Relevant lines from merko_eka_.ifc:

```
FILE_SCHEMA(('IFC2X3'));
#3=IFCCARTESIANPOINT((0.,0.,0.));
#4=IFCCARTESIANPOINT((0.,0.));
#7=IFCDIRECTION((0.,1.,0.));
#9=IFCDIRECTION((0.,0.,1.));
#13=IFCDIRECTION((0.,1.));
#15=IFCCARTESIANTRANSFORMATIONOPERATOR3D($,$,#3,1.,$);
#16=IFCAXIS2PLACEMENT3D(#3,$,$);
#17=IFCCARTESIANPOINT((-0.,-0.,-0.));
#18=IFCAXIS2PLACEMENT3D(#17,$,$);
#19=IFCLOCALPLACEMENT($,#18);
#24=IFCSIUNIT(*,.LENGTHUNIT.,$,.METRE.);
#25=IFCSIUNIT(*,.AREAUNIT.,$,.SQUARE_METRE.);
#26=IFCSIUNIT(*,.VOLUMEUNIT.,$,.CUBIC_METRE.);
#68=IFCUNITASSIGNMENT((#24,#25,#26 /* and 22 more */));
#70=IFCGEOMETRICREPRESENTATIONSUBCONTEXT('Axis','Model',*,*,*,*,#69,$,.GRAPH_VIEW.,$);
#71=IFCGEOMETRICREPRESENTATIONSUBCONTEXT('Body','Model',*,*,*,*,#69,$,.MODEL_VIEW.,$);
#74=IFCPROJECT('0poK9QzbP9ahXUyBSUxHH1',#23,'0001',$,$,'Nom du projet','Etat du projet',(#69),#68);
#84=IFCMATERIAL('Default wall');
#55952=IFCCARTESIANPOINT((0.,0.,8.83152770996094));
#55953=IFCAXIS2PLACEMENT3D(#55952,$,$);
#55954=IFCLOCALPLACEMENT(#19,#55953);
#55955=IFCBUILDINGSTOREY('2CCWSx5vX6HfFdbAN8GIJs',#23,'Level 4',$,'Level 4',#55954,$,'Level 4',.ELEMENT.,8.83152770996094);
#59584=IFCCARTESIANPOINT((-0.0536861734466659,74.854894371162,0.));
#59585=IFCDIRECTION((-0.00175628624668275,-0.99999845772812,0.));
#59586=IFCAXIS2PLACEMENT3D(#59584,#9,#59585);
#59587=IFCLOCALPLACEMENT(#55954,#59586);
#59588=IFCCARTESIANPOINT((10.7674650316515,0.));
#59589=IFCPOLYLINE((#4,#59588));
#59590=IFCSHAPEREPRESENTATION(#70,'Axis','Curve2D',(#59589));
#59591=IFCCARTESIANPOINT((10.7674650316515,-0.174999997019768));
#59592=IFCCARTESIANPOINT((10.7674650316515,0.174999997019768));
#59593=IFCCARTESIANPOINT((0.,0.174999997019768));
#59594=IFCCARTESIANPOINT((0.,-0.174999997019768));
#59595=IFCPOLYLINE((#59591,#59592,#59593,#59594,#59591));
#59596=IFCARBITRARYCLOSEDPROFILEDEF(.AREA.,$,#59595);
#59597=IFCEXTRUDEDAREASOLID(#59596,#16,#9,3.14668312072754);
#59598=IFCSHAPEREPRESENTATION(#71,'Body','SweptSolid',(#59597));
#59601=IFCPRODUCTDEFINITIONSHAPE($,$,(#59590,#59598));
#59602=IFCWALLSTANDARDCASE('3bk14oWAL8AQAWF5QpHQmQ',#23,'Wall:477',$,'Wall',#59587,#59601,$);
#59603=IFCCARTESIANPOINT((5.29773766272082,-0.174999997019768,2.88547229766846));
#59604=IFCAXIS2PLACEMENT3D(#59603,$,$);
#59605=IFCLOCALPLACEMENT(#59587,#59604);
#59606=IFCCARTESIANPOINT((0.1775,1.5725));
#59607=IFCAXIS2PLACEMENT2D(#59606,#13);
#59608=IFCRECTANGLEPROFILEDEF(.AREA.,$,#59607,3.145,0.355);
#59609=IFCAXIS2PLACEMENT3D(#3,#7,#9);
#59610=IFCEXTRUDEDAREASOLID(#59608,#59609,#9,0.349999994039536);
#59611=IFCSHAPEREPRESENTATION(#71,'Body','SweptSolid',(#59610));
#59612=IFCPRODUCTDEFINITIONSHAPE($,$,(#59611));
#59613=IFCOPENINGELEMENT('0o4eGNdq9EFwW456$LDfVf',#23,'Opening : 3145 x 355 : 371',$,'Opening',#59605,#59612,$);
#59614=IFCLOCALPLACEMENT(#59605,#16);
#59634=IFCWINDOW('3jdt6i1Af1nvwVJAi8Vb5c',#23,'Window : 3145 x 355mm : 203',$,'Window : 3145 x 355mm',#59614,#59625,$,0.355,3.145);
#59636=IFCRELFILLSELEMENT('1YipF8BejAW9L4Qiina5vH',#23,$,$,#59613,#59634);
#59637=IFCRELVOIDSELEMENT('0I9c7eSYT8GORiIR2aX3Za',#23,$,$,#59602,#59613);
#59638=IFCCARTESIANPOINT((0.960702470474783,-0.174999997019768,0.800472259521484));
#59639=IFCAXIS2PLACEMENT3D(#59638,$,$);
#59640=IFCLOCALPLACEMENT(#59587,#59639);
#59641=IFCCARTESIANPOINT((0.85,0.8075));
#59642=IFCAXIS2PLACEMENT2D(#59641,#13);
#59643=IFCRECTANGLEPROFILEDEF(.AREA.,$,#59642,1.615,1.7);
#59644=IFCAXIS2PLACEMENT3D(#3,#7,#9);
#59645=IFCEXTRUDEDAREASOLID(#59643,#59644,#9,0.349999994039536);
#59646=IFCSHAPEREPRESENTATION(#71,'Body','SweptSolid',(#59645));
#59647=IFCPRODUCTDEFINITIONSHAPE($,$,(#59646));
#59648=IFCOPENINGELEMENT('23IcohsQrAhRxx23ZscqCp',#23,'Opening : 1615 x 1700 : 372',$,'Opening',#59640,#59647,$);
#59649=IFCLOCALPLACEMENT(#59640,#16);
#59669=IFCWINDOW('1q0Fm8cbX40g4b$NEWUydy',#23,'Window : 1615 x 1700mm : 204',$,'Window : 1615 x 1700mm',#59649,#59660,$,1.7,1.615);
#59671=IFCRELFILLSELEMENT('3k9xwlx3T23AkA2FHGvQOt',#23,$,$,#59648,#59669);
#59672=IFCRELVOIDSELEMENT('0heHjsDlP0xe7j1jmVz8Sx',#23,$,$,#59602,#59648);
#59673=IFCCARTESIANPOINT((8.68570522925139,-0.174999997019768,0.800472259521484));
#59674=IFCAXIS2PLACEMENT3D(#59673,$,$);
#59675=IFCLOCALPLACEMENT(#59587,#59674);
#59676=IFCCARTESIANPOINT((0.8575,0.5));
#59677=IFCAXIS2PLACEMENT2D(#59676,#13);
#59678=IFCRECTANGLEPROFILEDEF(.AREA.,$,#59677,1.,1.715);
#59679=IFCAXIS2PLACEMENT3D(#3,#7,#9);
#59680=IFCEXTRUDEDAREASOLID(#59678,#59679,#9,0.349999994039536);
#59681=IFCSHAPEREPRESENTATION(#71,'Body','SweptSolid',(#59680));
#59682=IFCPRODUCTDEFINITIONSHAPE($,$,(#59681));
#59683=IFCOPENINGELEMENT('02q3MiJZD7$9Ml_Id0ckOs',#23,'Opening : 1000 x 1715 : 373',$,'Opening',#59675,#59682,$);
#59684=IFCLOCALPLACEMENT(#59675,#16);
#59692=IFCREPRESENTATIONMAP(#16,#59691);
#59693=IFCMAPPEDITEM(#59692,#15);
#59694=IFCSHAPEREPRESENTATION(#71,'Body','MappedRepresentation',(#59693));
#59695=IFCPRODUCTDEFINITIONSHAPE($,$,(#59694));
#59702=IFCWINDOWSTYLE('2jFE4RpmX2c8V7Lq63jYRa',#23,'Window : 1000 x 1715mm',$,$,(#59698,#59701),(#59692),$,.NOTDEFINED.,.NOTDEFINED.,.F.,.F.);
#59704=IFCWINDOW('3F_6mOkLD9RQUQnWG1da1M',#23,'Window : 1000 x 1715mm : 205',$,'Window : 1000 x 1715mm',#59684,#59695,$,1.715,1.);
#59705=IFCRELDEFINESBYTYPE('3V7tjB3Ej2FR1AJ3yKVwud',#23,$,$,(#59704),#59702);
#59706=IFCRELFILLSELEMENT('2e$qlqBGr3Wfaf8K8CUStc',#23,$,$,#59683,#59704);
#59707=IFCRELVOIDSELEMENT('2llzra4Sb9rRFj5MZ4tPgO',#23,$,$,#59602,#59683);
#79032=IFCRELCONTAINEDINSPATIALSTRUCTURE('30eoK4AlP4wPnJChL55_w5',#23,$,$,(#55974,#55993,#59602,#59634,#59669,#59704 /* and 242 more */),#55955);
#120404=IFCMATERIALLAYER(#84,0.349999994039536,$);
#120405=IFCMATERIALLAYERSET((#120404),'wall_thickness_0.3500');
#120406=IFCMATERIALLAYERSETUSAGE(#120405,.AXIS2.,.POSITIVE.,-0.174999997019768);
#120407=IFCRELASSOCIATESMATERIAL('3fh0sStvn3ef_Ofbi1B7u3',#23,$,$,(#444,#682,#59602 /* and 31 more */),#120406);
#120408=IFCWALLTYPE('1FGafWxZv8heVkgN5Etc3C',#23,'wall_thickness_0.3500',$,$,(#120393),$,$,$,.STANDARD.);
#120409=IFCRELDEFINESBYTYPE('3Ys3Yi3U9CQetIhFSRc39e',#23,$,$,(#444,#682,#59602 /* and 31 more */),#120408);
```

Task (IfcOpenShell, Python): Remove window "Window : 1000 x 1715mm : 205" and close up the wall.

```python
import ifcopenshell
import ifcopenshell.api.feature
import ifcopenshell.api.root
import ifcopenshell.geom
import ifcopenshell.util.shape

model = ifcopenshell.open("merko_eka_.ifc")
settings = ifcopenshell.geom.settings()


def volume(element):
    """Net volume in cubic metres, openings subtracted."""
    shape = ifcopenshell.geom.create_shape(settings, element)
    return ifcopenshell.util.shape.get_volume(shape.geometry)


window = model.by_guid("3F_6mOkLD9RQUQnWG1da1M")
opening = window.FillsVoids[0].RelatingOpeningElement
wall = opening.VoidsElements[0].RelatingBuildingElement
before = volume(wall)

ifcopenshell.api.root.remove_product(model, product=window)
ifcopenshell.api.feature.remove_feature(model, feature=opening)

after = volume(wall)

print(f"wall volume {before:.3f} -> {after:.3f} m3")

model.write("merko_eka__v2.ifc")
```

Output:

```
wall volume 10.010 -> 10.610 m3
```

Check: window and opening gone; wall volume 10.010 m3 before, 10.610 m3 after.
